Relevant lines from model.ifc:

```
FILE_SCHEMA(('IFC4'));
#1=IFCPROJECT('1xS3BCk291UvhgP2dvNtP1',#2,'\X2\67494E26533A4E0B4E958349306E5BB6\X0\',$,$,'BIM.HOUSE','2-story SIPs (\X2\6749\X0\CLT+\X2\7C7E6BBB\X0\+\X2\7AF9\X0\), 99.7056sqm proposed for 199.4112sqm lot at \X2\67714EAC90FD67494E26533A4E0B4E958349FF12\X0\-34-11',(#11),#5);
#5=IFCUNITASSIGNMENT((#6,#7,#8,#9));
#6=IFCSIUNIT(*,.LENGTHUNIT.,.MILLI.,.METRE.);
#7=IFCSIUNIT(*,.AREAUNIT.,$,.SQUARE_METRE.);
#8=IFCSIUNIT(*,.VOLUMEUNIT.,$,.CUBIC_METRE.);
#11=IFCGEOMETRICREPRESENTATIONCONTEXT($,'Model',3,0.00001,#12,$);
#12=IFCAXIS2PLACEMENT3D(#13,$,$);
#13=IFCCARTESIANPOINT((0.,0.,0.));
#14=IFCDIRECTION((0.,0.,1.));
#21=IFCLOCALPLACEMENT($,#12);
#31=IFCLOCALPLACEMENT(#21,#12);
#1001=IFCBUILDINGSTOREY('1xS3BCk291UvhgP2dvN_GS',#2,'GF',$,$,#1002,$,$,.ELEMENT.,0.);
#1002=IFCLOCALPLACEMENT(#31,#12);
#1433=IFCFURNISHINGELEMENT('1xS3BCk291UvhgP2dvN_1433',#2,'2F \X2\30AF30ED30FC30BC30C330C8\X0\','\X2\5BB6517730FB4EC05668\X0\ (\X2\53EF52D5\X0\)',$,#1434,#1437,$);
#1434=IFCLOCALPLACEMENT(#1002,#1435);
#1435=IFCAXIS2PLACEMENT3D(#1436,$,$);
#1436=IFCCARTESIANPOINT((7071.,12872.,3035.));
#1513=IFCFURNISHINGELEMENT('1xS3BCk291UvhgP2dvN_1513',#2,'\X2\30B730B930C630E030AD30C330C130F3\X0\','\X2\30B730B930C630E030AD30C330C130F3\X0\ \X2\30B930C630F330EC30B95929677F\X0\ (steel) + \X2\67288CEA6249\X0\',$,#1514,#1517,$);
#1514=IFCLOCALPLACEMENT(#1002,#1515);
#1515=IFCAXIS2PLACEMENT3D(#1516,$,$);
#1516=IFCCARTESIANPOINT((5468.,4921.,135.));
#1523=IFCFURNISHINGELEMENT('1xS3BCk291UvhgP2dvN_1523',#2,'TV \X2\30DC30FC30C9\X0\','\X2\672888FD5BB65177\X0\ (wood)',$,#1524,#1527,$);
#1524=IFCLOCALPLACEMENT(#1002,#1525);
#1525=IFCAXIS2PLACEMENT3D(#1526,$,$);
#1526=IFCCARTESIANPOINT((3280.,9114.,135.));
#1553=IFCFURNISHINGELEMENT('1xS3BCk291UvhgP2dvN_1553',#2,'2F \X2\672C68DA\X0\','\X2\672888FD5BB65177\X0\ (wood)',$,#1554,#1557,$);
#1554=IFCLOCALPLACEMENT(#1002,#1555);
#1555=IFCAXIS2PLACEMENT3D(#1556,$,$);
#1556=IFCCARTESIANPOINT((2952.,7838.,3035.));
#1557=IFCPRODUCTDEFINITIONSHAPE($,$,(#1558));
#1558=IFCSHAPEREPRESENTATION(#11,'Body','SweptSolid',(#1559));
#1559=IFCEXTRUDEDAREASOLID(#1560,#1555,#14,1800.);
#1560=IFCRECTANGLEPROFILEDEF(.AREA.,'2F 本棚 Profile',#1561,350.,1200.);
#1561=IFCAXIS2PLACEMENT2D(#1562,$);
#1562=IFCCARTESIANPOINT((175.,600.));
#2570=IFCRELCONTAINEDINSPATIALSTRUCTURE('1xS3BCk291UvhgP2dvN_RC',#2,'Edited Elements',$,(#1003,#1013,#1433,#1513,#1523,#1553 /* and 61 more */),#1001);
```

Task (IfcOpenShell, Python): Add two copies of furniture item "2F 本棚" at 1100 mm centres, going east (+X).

```python
import numpy as np
import ifcopenshell
import ifcopenshell.api.geometry
import ifcopenshell.api.root
import ifcopenshell.util.element
import ifcopenshell.util.placement
import ifcopenshell.util.unit

model = ifcopenshell.open("model.ifc")
unit_scale = ifcopenshell.util.unit.calculate_unit_scale(model)


def reuse_history(source, copy):
    """copy_class also copies each property set's owner history, people and application; keep the originals."""
    for rel in copy.IsDefinedBy:
        if rel.is_a("IfcRelDefinesByProperties") and (history := rel.RelatingPropertyDefinition.OwnerHistory):
            rel.RelatingPropertyDefinition.OwnerHistory = source.OwnerHistory
            ifcopenshell.util.element.remove_deep2(model, history)


source = model.by_guid("1xS3BCk291UvhgP2dvN_1553")
base = ifcopenshell.util.placement.get_local_placement(source.ObjectPlacement)
step = np.array([1.0, 0.0, 0.0]) * 1.1 / unit_scale

for i in range(1, 3):
    copy = ifcopenshell.api.root.copy_class(model, product=source)
    copy.Representation = ifcopenshell.util.element.copy_deep(
        model, source.Representation, exclude=["IfcGeometricRepresentationContext", "IfcRepresentationMap"]
    )
    reuse_history(source, copy)
    matrix = base.copy()
    matrix[:3, 3] += i * step
    print("added at", matrix[:3, 3].round(3) + 0.0)
    ifcopenshell.api.geometry.edit_object_placement(model, product=copy, matrix=matrix, is_si=False)

model.write("model_rev.ifc")
```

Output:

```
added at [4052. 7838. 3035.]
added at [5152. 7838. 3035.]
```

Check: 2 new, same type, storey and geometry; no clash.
